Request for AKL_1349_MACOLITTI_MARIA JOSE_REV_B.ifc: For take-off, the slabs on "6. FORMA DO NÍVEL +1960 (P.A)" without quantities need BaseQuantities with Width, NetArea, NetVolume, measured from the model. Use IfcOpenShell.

First a look at what the model holds.

```python
import ifcopenshell
import ifcopenshell.util.element
import ifcopenshell.util.unit

model = ifcopenshell.open("AKL_1349_MACOLITTI_MARIA JOSE_REV_B.ifc")
print(model.schema)
for unit_type in ("LENGTHUNIT", "AREAUNIT", "VOLUMEUNIT"):
    print(unit_type, ifcopenshell.util.unit.calculate_unit_scale(model, unit_type))
storey = next(s for s in model.by_type("IfcBuildingStorey") if s.Name == "6. FORMA DO NÍVEL +1960 (P.A)")
slabs = [e for e in ifcopenshell.util.element.get_decomposition(storey) if e.is_a("IfcSlab")]
for e in sorted(slabs, key=lambda e: e.id()):
    print(e.id(), e.is_a(), e.Name, list(ifcopenshell.util.element.get_psets(e, qtos_only=True)), sep=" | ")
```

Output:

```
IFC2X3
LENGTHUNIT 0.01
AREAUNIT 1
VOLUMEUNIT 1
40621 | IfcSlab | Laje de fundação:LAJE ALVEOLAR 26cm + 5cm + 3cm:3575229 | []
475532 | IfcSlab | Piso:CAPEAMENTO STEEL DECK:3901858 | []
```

```python
import ifcopenshell
import ifcopenshell.api.pset
import ifcopenshell.geom
import ifcopenshell.util.element
import ifcopenshell.util.shape
import ifcopenshell.util.unit

model = ifcopenshell.open("AKL_1349_MACOLITTI_MARIA JOSE_REV_B.ifc")
unit_scale = ifcopenshell.util.unit.calculate_unit_scale(model)
area_scale = ifcopenshell.util.unit.calculate_unit_scale(model, "AREAUNIT")
volume_scale = ifcopenshell.util.unit.calculate_unit_scale(model, "VOLUMEUNIT")
settings = ifcopenshell.geom.settings()

storey = next(s for s in model.by_type("IfcBuildingStorey") if s.Name == "6. FORMA DO NÍVEL +1960 (P.A)")
slabs = [e for e in ifcopenshell.util.element.get_decomposition(storey) if e.is_a("IfcSlab")]

for e in sorted(slabs, key=lambda e: e.id()):
    if ifcopenshell.util.element.get_psets(e, qtos_only=True, should_inherit=False):
        continue
    # Geometry comes back in metres, in the element's own axes.
    shape = ifcopenshell.geom.create_shape(settings, e)
    values = {
        "Width": ifcopenshell.util.shape.get_z(shape.geometry) / unit_scale,
        "NetArea": ifcopenshell.util.shape.get_footprint_area(shape.geometry) / area_scale,
        "NetVolume": ifcopenshell.util.shape.get_volume(shape.geometry) / volume_scale,
    }
    qto = ifcopenshell.api.pset.add_qto(model, product=e, name="BaseQuantities")
    ifcopenshell.api.pset.edit_qto(model, qto=qto, properties=values)
    print(e.id(), {k: round(v, 3) for k, v in values.items()})

model.write("AKL_1349_MACOLITTI_MARIA JOSE_REV_B-out.ifc")
```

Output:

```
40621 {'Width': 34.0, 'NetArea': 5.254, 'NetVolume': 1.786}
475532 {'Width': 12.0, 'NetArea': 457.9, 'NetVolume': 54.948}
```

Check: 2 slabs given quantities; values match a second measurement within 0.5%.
